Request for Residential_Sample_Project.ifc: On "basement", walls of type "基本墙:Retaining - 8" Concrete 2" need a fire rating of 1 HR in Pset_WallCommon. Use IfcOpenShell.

First a look at what the model holds.

```python
import ifcopenshell
import ifcopenshell.util.element

model = ifcopenshell.open("Residential_Sample_Project.ifc")
print(model.schema)
storey = next(s for s in model.by_type("IfcBuildingStorey") if s.Name == "basement")
walls = [e for e in ifcopenshell.util.element.get_decomposition(storey) if e.is_a("IfcWall")]
seen = {}
for e in walls:
    element_type = ifcopenshell.util.element.get_type(e)
    key = (element_type.Name if element_type != e and element_type else None, ifcopenshell.util.element.get_pset(e, "Pset_WallCommon", "FireRating"))
    seen[key] = seen.get(key, 0) + 1
for (name, value), count in sorted(seen.items(), key=str):
    print(count, "x", name, "|", value)
```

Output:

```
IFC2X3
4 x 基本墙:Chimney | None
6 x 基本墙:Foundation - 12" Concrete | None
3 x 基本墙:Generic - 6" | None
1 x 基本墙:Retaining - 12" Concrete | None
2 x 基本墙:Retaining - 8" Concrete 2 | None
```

```python
import ifcopenshell
import ifcopenshell.api.pset
import ifcopenshell.util.element

model = ifcopenshell.open("Residential_Sample_Project.ifc")

storey = next(s for s in model.by_type("IfcBuildingStorey") if s.Name == "basement")
walls = [e for e in ifcopenshell.util.element.get_decomposition(storey) if e.is_a("IfcWall")]

count = 0
for e in walls:
    element_type = ifcopenshell.util.element.get_type(e)
    if element_type in (None, e) or element_type.Name != '基本墙:Retaining - 8" Concrete 2':
        continue
    # add_pset returns the element's existing set when there is one.
    pset = ifcopenshell.api.pset.add_pset(model, product=e, name="Pset_WallCommon")
    ifcopenshell.api.pset.edit_pset(model, pset=pset, properties={"FireRating": "1 HR"})
    count += 1

print(count, "walls updated")

model.write("Residential_Sample_Project_v2.ifc")
```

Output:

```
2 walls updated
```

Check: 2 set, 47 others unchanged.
